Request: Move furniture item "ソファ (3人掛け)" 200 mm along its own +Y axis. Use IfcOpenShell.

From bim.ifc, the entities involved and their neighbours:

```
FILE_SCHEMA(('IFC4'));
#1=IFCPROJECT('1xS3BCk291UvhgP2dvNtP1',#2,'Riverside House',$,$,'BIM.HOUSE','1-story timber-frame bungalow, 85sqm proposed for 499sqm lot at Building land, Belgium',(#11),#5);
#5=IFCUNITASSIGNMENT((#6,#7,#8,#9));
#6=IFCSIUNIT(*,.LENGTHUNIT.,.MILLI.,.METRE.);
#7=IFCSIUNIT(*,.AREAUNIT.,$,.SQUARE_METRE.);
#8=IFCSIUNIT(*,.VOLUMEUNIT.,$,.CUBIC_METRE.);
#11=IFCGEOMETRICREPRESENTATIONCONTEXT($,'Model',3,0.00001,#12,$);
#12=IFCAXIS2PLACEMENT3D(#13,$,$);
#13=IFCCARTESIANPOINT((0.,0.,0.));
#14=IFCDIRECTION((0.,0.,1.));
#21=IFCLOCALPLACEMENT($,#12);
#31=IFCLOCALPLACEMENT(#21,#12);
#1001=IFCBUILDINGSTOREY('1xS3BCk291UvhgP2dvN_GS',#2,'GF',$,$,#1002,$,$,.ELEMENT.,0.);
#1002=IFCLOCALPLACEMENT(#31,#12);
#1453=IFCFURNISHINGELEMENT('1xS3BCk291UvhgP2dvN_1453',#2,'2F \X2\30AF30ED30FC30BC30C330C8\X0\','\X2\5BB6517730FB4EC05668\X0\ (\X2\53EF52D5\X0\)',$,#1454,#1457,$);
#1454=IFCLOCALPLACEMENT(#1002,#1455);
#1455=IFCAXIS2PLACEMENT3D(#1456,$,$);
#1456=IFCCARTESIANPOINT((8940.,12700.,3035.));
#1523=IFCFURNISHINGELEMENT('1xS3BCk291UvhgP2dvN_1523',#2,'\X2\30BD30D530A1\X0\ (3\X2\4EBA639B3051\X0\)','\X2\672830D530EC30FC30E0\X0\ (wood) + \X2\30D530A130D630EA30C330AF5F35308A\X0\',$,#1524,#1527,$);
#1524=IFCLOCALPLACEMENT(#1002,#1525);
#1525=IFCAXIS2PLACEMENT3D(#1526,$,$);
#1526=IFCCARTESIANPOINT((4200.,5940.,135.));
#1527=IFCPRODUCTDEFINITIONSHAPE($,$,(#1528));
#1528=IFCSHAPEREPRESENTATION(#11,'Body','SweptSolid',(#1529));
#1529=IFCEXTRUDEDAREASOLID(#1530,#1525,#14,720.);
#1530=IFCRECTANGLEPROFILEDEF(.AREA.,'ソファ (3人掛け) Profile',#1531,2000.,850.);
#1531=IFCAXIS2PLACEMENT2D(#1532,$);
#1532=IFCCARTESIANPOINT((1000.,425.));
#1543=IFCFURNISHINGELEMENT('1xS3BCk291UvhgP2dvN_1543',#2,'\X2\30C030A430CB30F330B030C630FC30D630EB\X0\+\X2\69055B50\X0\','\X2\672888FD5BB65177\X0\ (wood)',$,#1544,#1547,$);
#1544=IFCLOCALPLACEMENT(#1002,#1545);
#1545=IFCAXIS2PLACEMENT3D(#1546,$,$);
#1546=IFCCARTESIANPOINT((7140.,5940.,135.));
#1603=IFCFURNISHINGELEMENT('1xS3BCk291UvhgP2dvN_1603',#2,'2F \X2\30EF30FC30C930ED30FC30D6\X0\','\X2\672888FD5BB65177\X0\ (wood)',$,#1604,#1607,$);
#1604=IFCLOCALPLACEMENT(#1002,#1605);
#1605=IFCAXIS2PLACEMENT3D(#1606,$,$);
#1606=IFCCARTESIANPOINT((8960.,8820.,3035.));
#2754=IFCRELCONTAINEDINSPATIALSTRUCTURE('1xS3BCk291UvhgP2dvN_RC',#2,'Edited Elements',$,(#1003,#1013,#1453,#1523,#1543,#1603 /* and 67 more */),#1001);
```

```python
import ifcopenshell
import ifcopenshell.api.geometry
import ifcopenshell.util.placement

model = ifcopenshell.open("bim.ifc")

item = model.by_guid("1xS3BCk291UvhgP2dvN_1523")
matrix = ifcopenshell.util.placement.get_local_placement(item.ObjectPlacement)
matrix[:3, 3] += matrix[:3, 1] * 200.0
ifcopenshell.api.geometry.edit_object_placement(model, product=item, matrix=matrix, is_si=False)

print(ifcopenshell.util.placement.get_local_placement(item.ObjectPlacement).round(3) + 0.0)

model.write("bim_edited.ifc")
```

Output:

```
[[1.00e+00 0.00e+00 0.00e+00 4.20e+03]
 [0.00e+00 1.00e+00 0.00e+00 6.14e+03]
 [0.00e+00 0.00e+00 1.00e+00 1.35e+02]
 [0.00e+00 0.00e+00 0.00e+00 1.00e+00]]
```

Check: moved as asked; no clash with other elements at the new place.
